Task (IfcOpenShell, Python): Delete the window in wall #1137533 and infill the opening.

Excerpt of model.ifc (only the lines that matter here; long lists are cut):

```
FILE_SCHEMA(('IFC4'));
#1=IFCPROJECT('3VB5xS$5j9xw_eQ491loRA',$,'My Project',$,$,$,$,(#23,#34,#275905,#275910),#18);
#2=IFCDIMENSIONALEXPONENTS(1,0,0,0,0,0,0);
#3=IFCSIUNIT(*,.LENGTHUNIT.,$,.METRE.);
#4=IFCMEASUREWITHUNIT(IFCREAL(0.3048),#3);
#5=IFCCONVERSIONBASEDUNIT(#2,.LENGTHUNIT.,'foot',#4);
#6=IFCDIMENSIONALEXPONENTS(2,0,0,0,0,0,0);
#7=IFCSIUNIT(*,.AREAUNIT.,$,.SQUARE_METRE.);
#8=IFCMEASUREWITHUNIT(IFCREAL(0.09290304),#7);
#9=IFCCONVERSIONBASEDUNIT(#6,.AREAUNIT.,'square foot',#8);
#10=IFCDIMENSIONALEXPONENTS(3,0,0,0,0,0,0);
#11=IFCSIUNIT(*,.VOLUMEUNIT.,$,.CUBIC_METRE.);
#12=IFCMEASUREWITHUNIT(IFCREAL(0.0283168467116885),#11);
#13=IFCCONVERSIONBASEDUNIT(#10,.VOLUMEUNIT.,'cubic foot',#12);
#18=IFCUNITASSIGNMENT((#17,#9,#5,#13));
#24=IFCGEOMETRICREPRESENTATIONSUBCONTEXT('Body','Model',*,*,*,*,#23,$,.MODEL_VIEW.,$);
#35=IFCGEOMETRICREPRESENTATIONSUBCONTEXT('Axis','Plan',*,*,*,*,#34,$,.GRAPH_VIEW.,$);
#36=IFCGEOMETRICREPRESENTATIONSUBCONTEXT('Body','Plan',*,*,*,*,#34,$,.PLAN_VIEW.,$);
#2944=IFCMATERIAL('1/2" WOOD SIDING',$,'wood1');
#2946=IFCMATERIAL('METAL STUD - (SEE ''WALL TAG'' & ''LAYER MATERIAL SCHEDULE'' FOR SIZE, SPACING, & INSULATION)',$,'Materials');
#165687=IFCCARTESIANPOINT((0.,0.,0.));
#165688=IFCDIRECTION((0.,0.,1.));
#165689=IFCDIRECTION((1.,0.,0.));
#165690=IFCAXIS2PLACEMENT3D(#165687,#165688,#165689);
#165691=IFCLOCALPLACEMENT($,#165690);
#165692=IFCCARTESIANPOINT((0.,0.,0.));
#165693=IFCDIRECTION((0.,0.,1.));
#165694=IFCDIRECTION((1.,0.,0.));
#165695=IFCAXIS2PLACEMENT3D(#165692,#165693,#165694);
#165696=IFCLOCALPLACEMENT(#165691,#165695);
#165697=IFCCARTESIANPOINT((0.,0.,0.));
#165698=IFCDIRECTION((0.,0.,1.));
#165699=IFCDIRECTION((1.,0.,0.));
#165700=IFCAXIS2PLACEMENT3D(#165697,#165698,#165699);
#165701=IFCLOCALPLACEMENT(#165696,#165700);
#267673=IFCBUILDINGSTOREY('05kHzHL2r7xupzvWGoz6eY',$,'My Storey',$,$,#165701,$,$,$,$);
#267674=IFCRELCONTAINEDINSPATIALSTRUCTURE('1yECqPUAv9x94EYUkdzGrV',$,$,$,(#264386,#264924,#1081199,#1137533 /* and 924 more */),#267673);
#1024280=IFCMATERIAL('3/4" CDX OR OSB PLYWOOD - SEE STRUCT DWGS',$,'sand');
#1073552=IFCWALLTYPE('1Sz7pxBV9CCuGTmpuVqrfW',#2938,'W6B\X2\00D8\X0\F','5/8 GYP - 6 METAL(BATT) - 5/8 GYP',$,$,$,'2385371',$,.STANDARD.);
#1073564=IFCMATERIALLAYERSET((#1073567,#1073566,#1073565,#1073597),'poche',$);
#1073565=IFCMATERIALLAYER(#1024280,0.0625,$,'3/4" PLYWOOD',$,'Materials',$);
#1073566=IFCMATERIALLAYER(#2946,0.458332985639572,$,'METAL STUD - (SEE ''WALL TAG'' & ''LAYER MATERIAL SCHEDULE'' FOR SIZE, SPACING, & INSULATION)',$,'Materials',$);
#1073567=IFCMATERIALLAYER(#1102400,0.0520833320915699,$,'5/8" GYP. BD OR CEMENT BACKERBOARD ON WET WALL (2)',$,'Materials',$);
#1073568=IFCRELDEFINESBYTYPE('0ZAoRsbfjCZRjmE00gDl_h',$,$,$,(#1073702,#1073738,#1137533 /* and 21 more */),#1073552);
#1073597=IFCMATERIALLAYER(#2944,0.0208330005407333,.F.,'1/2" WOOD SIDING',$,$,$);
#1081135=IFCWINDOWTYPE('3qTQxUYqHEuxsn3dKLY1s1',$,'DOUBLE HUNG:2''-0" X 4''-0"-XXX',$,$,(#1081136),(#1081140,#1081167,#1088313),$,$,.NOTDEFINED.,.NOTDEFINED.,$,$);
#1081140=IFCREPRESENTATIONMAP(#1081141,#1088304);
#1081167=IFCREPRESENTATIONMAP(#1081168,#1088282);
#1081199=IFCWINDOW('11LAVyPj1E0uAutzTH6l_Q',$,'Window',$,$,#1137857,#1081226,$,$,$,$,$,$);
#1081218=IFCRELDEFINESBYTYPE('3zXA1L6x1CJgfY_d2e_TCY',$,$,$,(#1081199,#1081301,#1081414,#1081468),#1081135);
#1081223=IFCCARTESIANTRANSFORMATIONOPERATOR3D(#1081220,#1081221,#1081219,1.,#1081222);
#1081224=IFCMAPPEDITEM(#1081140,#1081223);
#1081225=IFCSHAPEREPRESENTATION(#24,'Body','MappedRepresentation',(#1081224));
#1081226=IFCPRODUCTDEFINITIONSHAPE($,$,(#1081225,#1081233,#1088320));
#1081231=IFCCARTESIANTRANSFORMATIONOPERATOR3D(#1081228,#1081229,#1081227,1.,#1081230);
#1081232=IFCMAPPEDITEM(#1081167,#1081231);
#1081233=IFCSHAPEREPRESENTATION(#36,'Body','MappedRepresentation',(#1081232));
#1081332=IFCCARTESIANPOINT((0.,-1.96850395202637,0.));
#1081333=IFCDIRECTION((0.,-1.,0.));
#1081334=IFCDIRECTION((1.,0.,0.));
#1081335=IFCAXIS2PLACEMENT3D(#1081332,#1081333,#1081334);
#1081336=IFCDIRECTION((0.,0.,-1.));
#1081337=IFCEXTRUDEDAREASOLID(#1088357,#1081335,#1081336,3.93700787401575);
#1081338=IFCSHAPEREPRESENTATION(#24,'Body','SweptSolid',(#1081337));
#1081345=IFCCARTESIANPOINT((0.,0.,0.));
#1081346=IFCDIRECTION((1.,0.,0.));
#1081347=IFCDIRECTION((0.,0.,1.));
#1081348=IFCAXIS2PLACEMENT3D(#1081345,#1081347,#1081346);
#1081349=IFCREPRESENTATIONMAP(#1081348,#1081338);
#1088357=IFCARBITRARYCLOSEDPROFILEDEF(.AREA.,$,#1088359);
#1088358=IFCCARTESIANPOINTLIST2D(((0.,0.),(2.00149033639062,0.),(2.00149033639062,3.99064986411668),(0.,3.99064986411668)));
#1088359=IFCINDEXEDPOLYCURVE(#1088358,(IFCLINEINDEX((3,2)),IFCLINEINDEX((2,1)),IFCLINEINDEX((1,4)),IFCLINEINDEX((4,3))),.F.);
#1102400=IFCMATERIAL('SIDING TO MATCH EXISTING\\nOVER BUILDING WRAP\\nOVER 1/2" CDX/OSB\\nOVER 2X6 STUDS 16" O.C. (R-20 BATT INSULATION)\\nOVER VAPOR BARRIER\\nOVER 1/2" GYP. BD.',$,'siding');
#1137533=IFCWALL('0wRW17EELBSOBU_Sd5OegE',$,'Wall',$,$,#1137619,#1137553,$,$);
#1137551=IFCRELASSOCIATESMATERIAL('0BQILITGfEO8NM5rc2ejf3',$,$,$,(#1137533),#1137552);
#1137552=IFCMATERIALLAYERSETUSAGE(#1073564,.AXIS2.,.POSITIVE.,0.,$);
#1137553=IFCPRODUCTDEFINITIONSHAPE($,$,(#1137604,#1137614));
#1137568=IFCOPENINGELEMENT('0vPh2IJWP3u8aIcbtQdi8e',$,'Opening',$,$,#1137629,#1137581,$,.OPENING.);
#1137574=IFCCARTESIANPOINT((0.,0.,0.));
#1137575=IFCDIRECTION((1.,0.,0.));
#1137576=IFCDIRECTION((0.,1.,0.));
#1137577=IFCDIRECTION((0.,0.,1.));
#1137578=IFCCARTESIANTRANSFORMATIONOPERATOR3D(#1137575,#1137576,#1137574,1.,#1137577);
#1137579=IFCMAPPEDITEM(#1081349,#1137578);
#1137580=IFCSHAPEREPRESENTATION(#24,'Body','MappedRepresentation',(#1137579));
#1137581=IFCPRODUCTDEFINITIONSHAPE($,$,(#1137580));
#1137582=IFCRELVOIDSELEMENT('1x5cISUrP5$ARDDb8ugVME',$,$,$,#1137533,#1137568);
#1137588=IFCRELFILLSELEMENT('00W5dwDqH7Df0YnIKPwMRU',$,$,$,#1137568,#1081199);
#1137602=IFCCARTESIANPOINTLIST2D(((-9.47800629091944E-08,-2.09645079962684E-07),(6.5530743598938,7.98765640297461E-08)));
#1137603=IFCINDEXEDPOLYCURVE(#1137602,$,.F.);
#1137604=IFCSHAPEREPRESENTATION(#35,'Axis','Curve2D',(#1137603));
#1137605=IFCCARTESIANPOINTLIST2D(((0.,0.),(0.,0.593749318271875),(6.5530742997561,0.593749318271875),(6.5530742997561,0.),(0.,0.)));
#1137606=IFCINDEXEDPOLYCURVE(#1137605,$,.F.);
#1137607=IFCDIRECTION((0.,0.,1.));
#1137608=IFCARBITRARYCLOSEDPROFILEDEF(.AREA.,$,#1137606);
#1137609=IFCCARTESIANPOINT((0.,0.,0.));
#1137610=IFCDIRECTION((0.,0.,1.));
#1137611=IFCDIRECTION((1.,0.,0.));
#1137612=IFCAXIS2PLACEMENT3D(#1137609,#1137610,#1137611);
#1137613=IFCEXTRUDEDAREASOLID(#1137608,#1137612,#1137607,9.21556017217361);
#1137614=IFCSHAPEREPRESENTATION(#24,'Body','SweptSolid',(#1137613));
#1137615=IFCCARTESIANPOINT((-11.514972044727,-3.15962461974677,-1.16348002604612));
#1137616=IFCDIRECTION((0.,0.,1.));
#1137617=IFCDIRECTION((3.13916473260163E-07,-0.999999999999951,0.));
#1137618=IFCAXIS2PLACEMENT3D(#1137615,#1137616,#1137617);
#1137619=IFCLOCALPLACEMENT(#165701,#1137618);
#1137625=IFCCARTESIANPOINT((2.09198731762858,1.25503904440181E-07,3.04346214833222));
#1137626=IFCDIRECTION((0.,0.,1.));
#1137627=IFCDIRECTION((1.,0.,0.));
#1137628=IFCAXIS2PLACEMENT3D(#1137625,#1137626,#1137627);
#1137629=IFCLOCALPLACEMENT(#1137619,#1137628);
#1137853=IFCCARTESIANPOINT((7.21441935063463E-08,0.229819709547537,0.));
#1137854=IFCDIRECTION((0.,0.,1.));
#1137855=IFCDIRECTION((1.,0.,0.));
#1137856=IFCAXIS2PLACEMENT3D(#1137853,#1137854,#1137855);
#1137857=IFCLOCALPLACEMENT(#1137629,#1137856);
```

```python
import ifcopenshell
import ifcopenshell.api.feature
import ifcopenshell.api.root
import ifcopenshell.geom
import ifcopenshell.util.shape

model = ifcopenshell.open("model.ifc")
settings = ifcopenshell.geom.settings()


def volume(element):
    """Net volume in cubic metres, openings subtracted."""
    shape = ifcopenshell.geom.create_shape(settings, element)
    return ifcopenshell.util.shape.get_volume(shape.geometry)


window = model.by_id(1081199)
opening = window.FillsVoids[0].RelatingOpeningElement
wall = opening.VoidsElements[0].RelatingBuildingElement
before = volume(wall)

ifcopenshell.api.root.remove_product(model, product=window)
ifcopenshell.api.feature.remove_feature(model, feature=opening)

after = volume(wall)

print(f"wall volume {before:.3f} -> {after:.3f} m3")

model.write("model_edited.ifc")
```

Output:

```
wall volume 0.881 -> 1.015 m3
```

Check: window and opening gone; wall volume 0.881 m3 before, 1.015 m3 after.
